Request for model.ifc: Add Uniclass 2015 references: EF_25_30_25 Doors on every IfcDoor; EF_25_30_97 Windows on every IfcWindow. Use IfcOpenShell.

First a look at what the model holds.

```python
import ifcopenshell

model = ifcopenshell.open("model.ifc")
print(model.schema)
print("classifications:", [c.Name for c in model.by_type("IfcClassification")])
for ifc_class in ("IfcDoor", "IfcRoof", "IfcStair", "IfcWall", "IfcWindow"):
    print(ifc_class, len(model.by_type(ifc_class)))
```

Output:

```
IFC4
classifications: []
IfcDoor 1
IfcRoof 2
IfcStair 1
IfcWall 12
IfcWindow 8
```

```python
import ifcopenshell
import ifcopenshell.api.classification

model = ifcopenshell.open("model.ifc")

system = ifcopenshell.api.classification.add_classification(model, classification="Uniclass 2015")

codes = {
    "IfcDoor": ("EF_25_30_25", "Doors"),
    "IfcWindow": ("EF_25_30_97", "Windows"),
}
for ifc_class, (code, name) in codes.items():
    products = model.by_type(ifc_class)
    ifcopenshell.api.classification.add_reference(
        model, products=products, classification=system, identification=code, name=name
    )
    print(code, len(products))

model.write("model_v2.ifc")
```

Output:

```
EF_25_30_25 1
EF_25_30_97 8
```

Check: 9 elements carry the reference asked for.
